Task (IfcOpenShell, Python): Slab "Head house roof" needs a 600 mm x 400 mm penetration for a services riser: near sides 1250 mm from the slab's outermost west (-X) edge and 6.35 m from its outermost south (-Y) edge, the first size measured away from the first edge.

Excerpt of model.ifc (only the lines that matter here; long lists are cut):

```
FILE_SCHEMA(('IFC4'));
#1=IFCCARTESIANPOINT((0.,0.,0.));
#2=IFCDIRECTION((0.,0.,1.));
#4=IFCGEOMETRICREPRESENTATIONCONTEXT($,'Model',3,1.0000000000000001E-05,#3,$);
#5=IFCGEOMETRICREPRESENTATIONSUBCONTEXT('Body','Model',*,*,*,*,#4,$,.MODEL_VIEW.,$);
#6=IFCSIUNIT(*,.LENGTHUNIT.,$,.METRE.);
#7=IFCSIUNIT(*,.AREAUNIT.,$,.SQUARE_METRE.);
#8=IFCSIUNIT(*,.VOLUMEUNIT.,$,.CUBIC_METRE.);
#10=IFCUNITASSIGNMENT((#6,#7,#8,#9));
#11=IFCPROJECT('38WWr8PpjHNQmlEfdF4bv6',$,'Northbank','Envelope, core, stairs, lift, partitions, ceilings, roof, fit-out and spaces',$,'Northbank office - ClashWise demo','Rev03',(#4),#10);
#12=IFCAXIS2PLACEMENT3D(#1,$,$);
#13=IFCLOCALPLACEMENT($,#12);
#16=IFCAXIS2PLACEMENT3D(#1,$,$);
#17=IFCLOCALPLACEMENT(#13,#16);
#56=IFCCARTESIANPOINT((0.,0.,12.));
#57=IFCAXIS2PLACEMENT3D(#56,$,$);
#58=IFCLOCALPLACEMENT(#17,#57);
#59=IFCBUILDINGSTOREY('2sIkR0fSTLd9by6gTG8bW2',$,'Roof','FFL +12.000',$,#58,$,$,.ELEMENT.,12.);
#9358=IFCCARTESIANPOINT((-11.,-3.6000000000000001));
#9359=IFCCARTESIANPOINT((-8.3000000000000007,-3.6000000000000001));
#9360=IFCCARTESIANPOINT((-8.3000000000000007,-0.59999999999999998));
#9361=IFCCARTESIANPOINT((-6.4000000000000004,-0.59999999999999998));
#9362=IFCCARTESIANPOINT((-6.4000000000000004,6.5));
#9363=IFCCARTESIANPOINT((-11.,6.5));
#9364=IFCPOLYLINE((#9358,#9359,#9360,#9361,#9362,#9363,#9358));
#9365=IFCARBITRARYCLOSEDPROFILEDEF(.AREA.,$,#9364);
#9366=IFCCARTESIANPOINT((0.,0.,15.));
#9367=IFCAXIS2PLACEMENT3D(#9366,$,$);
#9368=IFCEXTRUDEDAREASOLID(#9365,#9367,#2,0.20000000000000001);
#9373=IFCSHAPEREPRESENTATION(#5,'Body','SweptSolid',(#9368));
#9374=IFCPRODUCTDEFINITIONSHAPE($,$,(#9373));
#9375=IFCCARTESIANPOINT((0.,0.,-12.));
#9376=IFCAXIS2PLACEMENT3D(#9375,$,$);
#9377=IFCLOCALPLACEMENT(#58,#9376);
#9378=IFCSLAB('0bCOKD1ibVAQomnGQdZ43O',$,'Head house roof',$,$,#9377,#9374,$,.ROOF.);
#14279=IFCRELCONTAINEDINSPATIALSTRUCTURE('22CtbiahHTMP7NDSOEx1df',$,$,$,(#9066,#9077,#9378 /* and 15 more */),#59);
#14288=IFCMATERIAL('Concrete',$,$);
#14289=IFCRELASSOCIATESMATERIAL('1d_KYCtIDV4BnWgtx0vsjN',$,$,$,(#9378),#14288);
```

```python
import numpy as np
import ifcopenshell
import ifcopenshell.api.feature
import ifcopenshell.api.geometry
import ifcopenshell.api.root
import ifcopenshell.geom
import ifcopenshell.util.placement
import ifcopenshell.util.representation
import ifcopenshell.util.shape
import ifcopenshell.util.unit

model = ifcopenshell.open("model.ifc")
unit_scale = ifcopenshell.util.unit.calculate_unit_scale(model)
settings = ifcopenshell.geom.settings()


def volume(element):
    """Net volume in cubic metres, openings subtracted."""
    shape = ifcopenshell.geom.create_shape(settings, element)
    return ifcopenshell.util.shape.get_volume(shape.geometry)


slab = model.by_guid("0bCOKD1ibVAQomnGQdZ43O")
before = volume(slab)

# Extent in the slab's own axes, in metres. The edges named are its -X and -Y sides.
slab_shape = ifcopenshell.geom.create_shape(settings, slab)
vertices = ifcopenshell.util.shape.get_vertices(slab_shape.geometry)
x_min, y_min, bottom = vertices.min(axis=0)
top = vertices[:, 2].max()

opening = ifcopenshell.api.root.create_entity(model, ifc_class="IfcOpeningElement", name="Services riser opening", predefined_type="OPENING")
context = ifcopenshell.util.representation.get_context(model, "Model", "Body", "MODEL_VIEW")
width, depth = 0.6, 0.4
outline = [(0.0, 0.0), (width, 0.0), (width, depth), (0.0, depth), (0.0, 0.0)]
# Overshoot both faces by 50 mm so the cut is clean.
shape = ifcopenshell.api.geometry.add_slab_representation(
    model, context=context, depth=top - bottom + 0.1, polyline=outline
)
ifcopenshell.api.geometry.assign_representation(model, product=opening, representation=shape)

matrix = ifcopenshell.util.placement.get_local_placement(slab.ObjectPlacement)
matrix[:, 3] = matrix @ np.append(np.array([x_min + 1.25, y_min + 6.35, bottom - 0.05]) / unit_scale, 1.0)
ifcopenshell.api.geometry.edit_object_placement(model, product=opening, matrix=matrix, is_si=False)
ifcopenshell.api.feature.add_feature(model, feature=opening, element=slab)

after = volume(slab)

print(f"slab volume {before:.3f} -> {after:.3f} m3")

model.write("model_updated.ifc")
```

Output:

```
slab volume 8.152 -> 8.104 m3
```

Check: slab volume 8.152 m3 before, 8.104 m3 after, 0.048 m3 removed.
